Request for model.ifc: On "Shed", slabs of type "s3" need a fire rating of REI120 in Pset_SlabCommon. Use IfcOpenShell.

First a look at what the model holds.

```python
import ifcopenshell
import ifcopenshell.util.element

model = ifcopenshell.open("model.ifc")
print(model.schema)
storey = next(s for s in model.by_type("IfcBuildingStorey") if s.Name == "Shed")
slabs = [e for e in ifcopenshell.util.element.get_decomposition(storey) if e.is_a("IfcSlab")]
seen = {}
for e in slabs:
    element_type = ifcopenshell.util.element.get_type(e)
    key = (element_type.Name if element_type != e and element_type else None, ifcopenshell.util.element.get_pset(e, "Pset_SlabCommon", "FireRating"))
    seen[key] = seen.get(key, 0) + 1
for (name, value), count in sorted(seen.items(), key=str):
    print(count, "x", name, "|", value)
```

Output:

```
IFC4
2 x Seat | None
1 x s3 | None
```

```python
import ifcopenshell
import ifcopenshell.api.pset
import ifcopenshell.util.element

model = ifcopenshell.open("model.ifc")

storey = next(s for s in model.by_type("IfcBuildingStorey") if s.Name == "Shed")
slabs = [e for e in ifcopenshell.util.element.get_decomposition(storey) if e.is_a("IfcSlab")]

count = 0
for e in slabs:
    element_type = ifcopenshell.util.element.get_type(e)
    if element_type in (None, e) or element_type.Name != "s3":
        continue
    # add_pset returns the element's existing set when there is one.
    pset = ifcopenshell.api.pset.add_pset(model, product=e, name="Pset_SlabCommon")
    ifcopenshell.api.pset.edit_pset(model, pset=pset, properties={"FireRating": "REI120"})
    count += 1

print(count, "slabs updated")

model.write("model-out.ifc")
```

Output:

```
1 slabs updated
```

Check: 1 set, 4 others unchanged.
